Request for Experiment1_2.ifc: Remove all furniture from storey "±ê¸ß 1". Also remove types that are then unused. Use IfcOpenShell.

First a look at what the model holds.

```python
import ifcopenshell
import ifcopenshell.util.element

model = ifcopenshell.open("Experiment1_2.ifc")
print(model.schema)
storey = next(s for s in model.by_type("IfcBuildingStorey") if s.Name == "±ê¸ß 1")
furniture = [e for e in ifcopenshell.util.element.get_decomposition(storey) if e.is_a("IfcFurnishingElement")]
seen = {}
for e in furniture:
    element_type = ifcopenshell.util.element.get_type(e)
    name = element_type.Name if element_type not in (None, e) else None
    seen[name] = seen.get(name, 0) + 1
for name, count in sorted(seen.items(), key=str):
    print(count, "x", name)
```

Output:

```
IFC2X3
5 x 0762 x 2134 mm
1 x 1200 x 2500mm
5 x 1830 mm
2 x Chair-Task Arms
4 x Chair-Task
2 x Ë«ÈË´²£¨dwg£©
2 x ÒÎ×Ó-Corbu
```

```python
import ifcopenshell
import ifcopenshell.api.root
import ifcopenshell.util.element

model = ifcopenshell.open("Experiment1_2.ifc")

storey = next(s for s in model.by_type("IfcBuildingStorey") if s.Name == "±ê¸ß 1")
furniture = [e for e in ifcopenshell.util.element.get_decomposition(storey) if e.is_a("IfcFurnishingElement")]
types = {ifcopenshell.util.element.get_type(e) for e in furniture} - {None, *furniture}

for e in furniture:
    ifcopenshell.api.root.remove_product(model, product=e)
print(len(furniture), "removed")

unused = [t for t in types if not ifcopenshell.util.element.get_types(t)]
for t in unused:
    ifcopenshell.api.root.remove_product(model, product=t)
print(len(unused), "unused types removed")

model.write("Experiment1_2_updated.ifc")
```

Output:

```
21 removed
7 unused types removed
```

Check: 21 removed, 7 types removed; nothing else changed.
